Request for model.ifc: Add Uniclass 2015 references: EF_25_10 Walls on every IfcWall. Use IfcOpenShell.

First a look at what the model holds.

```python
import ifcopenshell

model = ifcopenshell.open("model.ifc")
print(model.schema)
print("classifications:", [c.Name for c in model.by_type("IfcClassification")])
for ifc_class in ("IfcDoor", "IfcRoof", "IfcStair", "IfcWall", "IfcWindow"):
    print(ifc_class, len(model.by_type(ifc_class)))
```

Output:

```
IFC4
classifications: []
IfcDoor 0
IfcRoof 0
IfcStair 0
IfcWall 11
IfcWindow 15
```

```python
import ifcopenshell
import ifcopenshell.api.classification

model = ifcopenshell.open("model.ifc")

system = ifcopenshell.api.classification.add_classification(model, classification="Uniclass 2015")

codes = {
    "IfcWall": ("EF_25_10", "Walls"),
}
for ifc_class, (code, name) in codes.items():
    products = model.by_type(ifc_class)
    ifcopenshell.api.classification.add_reference(
        model, products=products, classification=system, identification=code, name=name
    )
    print(code, len(products))

model.write("model-out.ifc")
```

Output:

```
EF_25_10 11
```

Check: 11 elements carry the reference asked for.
